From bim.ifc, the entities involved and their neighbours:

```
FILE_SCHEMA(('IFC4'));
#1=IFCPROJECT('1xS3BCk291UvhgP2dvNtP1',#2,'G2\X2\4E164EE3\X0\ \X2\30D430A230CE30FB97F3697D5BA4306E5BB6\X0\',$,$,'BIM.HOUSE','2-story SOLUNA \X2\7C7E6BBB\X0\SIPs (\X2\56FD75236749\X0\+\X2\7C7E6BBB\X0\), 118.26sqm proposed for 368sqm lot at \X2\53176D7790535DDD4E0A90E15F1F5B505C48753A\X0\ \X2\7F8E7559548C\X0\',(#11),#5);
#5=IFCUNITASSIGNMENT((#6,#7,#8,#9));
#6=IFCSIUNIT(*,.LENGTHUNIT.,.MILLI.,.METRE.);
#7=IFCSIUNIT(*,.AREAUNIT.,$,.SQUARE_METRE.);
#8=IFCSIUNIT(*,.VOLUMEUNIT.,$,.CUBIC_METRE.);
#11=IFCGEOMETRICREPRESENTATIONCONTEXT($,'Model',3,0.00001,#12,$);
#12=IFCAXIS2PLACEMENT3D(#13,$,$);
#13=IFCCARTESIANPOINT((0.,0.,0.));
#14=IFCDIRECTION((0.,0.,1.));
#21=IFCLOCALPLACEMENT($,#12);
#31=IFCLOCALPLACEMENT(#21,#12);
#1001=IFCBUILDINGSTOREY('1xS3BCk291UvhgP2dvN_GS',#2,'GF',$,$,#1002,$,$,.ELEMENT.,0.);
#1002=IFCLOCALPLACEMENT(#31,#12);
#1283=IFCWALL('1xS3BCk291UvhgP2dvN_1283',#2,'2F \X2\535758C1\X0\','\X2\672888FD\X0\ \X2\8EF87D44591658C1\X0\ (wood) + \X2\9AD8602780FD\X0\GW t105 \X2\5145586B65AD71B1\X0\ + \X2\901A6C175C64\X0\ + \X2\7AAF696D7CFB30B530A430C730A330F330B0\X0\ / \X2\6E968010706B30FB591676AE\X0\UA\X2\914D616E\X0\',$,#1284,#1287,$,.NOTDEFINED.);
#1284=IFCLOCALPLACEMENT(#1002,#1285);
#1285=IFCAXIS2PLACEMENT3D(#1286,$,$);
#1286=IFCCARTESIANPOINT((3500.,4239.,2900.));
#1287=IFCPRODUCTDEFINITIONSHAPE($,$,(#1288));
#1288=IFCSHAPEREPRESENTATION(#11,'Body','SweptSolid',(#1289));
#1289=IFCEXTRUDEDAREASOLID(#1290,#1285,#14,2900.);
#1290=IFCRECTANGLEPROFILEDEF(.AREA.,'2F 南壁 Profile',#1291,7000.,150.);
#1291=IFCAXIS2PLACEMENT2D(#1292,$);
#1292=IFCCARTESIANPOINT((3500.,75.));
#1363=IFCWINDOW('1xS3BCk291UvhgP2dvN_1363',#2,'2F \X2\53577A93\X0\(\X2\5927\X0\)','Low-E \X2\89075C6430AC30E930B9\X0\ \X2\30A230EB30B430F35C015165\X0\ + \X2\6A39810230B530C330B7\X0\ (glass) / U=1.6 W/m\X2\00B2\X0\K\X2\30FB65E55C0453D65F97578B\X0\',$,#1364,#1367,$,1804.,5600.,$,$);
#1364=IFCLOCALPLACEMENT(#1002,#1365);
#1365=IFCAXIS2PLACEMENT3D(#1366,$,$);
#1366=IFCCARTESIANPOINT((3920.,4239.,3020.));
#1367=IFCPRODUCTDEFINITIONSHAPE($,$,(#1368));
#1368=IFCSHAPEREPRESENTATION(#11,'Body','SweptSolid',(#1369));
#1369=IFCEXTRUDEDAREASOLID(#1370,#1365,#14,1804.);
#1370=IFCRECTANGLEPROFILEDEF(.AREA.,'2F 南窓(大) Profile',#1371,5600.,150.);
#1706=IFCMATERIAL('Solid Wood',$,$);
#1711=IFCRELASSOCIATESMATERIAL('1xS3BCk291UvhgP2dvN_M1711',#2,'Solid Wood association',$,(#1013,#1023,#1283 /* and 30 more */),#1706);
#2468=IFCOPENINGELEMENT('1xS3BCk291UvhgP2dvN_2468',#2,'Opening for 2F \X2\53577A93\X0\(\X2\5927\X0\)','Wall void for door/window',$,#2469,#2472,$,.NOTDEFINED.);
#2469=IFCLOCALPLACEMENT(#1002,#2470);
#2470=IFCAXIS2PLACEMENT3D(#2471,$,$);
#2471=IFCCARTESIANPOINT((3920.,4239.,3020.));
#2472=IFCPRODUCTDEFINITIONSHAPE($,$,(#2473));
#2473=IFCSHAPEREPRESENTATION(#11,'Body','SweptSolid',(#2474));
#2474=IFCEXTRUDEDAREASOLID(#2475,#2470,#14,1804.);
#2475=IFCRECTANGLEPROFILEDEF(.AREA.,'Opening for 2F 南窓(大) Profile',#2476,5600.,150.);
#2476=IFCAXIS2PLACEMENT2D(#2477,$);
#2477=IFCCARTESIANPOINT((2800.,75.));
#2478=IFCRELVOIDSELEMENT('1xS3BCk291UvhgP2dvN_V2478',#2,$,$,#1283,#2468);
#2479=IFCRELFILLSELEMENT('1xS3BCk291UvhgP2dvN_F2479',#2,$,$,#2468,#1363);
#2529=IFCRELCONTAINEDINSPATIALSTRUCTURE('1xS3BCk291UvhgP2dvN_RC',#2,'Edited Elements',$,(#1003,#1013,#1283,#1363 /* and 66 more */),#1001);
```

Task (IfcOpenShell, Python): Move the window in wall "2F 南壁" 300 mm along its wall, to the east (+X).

```python
import ifcopenshell
import ifcopenshell.api.geometry
import ifcopenshell.util.placement
import ifcopenshell.util.unit

model = ifcopenshell.open("bim.ifc")
unit_scale = ifcopenshell.util.unit.calculate_unit_scale(model)

window = model.by_id(1363)
opening = window.FillsVoids[0].RelatingOpeningElement
wall = opening.VoidsElements[0].RelatingBuildingElement

wall_matrix = ifcopenshell.util.placement.get_local_placement(wall.ObjectPlacement)
shift = wall_matrix[:3, 0] * 0.3 / unit_scale
before = ifcopenshell.util.placement.get_local_placement(window.ObjectPlacement)[:3, 3].copy()

# The window is not placed relative to its opening, so move both.
for product in (opening, window):
    matrix = ifcopenshell.util.placement.get_local_placement(product.ObjectPlacement)
    matrix[:3, 3] += shift
    ifcopenshell.api.geometry.edit_object_placement(model, product=product, matrix=matrix, is_si=False)

after = ifcopenshell.util.placement.get_local_placement(window.ObjectPlacement)[:3, 3]
print("window moved by", (after - before).round(3) + 0.0)

model.write("bim_edited.ifc")
```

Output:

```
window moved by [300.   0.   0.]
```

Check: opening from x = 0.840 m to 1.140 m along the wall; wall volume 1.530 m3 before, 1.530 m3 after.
